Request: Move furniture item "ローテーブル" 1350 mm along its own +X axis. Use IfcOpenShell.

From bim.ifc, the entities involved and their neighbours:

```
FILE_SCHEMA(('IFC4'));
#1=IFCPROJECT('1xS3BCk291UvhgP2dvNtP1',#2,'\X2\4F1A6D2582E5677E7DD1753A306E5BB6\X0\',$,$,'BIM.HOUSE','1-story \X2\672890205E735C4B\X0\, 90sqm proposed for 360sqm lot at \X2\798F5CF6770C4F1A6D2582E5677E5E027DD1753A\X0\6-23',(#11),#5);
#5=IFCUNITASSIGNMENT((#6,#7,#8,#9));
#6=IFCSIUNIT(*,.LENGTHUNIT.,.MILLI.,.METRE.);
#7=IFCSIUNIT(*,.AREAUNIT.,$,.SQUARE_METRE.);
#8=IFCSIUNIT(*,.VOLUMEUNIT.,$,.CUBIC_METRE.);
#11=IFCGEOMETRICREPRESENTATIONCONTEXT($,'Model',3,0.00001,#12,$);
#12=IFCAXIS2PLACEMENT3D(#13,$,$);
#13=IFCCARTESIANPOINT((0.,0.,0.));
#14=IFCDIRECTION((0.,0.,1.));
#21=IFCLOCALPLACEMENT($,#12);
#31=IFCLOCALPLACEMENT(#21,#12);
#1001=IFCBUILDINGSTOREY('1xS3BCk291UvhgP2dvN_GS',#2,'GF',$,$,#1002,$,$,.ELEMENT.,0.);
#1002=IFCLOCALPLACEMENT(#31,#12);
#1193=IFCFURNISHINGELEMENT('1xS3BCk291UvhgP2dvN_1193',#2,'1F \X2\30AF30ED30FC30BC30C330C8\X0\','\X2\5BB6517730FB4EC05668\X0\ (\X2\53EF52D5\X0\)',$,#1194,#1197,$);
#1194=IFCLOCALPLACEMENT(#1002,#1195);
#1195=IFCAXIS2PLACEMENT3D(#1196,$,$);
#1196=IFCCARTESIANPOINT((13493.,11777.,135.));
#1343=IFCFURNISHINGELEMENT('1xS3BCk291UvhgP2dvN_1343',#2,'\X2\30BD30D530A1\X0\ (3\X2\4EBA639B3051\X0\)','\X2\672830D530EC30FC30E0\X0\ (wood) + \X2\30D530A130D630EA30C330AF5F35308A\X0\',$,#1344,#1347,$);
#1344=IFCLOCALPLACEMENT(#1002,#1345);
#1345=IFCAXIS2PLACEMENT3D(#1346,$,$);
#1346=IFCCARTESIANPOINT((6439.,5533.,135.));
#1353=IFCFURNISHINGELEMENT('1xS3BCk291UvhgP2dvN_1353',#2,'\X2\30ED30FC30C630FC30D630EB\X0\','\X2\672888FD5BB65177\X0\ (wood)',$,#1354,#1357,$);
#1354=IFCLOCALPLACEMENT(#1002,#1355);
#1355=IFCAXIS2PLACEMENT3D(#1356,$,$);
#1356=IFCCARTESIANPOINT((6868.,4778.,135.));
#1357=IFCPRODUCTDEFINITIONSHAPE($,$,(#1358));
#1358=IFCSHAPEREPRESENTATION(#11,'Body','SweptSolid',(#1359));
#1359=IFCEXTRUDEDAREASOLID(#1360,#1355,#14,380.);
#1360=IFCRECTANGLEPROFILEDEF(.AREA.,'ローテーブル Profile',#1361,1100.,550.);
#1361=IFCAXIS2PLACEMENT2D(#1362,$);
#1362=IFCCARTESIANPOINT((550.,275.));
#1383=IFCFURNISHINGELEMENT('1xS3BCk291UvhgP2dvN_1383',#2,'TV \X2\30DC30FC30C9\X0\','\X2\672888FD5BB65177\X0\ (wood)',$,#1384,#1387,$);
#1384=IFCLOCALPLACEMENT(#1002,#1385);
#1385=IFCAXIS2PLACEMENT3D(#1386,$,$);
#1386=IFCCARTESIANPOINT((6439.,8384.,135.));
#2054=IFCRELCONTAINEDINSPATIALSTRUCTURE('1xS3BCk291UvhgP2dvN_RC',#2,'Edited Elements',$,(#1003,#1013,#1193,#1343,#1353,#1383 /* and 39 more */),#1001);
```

```python
import ifcopenshell
import ifcopenshell.api.geometry
import ifcopenshell.util.placement

model = ifcopenshell.open("bim.ifc")

item = model.by_guid("1xS3BCk291UvhgP2dvN_1353")
matrix = ifcopenshell.util.placement.get_local_placement(item.ObjectPlacement)
matrix[:3, 3] += matrix[:3, 0] * 1350.0
ifcopenshell.api.geometry.edit_object_placement(model, product=item, matrix=matrix, is_si=False)

print(ifcopenshell.util.placement.get_local_placement(item.ObjectPlacement).round(3) + 0.0)

model.write("bim_v2.ifc")
```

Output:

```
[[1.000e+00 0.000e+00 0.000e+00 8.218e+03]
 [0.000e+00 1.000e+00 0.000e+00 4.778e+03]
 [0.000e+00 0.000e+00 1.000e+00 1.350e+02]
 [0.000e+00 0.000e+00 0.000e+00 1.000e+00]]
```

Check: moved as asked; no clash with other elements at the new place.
